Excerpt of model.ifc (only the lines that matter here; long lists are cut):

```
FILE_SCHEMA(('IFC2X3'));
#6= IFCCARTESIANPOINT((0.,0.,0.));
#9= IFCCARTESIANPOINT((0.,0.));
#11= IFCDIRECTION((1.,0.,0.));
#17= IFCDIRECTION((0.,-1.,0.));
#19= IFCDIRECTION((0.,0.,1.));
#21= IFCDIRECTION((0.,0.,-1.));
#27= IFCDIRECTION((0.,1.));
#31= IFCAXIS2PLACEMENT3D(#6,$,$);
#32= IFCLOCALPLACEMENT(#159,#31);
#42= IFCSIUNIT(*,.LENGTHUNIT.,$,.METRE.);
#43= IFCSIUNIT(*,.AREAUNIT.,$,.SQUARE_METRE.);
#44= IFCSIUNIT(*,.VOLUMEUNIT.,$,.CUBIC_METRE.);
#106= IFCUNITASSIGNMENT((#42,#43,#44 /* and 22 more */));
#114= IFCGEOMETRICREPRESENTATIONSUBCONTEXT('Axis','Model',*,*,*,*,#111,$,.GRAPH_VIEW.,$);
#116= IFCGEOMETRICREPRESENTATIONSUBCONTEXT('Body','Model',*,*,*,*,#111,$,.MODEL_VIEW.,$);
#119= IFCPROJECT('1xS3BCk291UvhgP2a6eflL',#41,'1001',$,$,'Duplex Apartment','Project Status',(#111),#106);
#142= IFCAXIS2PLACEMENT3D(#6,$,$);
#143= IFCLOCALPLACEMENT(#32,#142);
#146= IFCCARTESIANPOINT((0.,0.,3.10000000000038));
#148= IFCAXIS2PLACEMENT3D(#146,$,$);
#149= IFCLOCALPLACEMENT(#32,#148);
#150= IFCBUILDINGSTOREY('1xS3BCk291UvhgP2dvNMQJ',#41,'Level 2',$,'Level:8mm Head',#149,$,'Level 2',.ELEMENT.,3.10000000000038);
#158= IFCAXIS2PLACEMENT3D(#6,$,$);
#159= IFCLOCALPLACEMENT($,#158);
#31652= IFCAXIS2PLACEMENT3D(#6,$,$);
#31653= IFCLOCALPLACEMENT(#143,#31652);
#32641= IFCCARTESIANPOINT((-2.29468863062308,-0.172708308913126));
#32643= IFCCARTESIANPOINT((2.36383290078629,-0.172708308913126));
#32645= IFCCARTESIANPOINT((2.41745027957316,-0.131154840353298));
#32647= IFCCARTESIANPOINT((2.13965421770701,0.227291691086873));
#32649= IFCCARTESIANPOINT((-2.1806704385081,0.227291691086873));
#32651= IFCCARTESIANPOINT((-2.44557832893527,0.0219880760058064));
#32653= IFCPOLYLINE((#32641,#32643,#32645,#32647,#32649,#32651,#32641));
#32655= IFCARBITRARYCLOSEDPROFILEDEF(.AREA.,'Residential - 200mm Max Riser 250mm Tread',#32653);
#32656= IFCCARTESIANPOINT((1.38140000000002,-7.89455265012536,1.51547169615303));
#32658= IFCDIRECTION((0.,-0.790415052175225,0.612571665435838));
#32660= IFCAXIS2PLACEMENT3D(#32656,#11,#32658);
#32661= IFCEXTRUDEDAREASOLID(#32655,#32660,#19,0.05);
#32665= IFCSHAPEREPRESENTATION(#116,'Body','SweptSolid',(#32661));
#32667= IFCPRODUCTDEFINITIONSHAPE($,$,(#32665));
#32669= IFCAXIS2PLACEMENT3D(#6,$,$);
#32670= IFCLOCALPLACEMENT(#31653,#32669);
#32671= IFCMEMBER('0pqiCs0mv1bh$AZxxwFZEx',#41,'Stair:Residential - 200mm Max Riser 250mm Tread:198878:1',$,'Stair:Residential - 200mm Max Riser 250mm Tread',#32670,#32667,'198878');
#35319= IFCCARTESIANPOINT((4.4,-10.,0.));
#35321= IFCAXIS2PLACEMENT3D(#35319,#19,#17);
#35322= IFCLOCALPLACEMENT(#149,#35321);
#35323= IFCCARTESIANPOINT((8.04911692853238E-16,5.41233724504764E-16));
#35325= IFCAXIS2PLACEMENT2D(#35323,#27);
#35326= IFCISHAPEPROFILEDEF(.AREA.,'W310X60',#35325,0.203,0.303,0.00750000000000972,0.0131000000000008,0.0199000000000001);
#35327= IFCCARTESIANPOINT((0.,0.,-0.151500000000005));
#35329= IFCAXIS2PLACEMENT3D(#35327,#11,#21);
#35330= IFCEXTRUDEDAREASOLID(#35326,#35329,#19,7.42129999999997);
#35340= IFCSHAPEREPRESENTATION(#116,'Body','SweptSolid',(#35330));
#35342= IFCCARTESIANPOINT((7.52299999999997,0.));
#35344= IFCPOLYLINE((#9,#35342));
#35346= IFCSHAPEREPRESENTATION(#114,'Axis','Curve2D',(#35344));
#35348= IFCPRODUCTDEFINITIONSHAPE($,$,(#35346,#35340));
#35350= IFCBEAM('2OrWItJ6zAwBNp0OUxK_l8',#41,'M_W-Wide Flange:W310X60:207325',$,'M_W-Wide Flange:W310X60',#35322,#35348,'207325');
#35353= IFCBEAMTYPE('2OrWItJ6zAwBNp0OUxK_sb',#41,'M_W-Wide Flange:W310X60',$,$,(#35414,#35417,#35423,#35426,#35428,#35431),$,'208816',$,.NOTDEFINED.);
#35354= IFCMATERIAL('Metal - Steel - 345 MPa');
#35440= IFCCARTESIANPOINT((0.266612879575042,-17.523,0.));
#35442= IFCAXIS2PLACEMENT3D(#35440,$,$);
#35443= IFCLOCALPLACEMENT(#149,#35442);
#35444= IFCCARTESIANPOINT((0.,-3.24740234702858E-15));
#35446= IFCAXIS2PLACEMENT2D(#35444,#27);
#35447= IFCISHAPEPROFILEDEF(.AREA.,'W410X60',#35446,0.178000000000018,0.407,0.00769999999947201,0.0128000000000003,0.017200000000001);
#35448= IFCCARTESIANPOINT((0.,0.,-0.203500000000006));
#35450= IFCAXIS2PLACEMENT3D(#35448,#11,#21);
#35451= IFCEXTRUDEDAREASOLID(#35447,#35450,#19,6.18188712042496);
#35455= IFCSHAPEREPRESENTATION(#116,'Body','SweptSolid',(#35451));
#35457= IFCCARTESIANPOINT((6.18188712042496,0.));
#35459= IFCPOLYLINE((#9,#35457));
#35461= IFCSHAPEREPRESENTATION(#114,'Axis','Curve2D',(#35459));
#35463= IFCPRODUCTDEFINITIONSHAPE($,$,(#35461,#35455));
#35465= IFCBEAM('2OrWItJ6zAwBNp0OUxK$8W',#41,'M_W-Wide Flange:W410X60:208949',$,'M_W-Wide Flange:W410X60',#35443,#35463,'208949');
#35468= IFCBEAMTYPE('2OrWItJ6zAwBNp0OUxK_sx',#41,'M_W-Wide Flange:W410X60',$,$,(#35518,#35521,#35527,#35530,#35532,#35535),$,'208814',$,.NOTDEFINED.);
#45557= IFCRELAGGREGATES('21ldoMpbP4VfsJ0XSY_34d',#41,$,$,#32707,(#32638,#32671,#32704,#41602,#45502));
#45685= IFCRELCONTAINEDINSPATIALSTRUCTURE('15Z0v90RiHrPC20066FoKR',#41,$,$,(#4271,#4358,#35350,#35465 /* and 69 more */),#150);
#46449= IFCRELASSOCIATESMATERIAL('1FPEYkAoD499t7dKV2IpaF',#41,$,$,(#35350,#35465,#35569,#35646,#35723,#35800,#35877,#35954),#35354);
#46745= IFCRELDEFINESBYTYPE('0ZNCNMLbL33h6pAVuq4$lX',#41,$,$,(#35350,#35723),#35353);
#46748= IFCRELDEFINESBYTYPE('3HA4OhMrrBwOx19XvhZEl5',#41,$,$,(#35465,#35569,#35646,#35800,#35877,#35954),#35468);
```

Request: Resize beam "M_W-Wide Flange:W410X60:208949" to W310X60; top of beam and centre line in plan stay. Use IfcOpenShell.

```python
import ifcopenshell
import ifcopenshell.api.type
import ifcopenshell.util.element
import ifcopenshell.util.representation

model = ifcopenshell.open("model.ifc")

member = model.by_guid("2OrWItJ6zAwBNp0OUxK$8W")
source = next(p for p in model.by_type("IfcIShapeProfileDef") if p.ProfileName == "W310X60")

body = ifcopenshell.util.representation.get_representation(member, "Model", "Body")
solid = body.Items[0]
old_profile = solid.SweptArea

# Copy the section's sizes but keep this member's own profile position.
profile = ifcopenshell.util.element.copy(model, source)
# Profiles are centred, so shift by half the change in depth to hold the top.
shift = (old_profile.OverallDepth - profile.OverallDepth) / 2
x, y = old_profile.Position.Location.Coordinates
up = (-1.0, 0.0)  # upwards, in the solid's own plane
location = model.createIfcCartesianPoint((x + up[0] * shift, y + up[1] * shift))
profile.Position = model.createIfcAxis2Placement2D(location, old_profile.Position.RefDirection)
solid.SweptArea = profile
if not model.get_total_inverses(old_profile):
    ifcopenshell.util.element.remove_deep2(model, old_profile)

new_type = model.by_id(35353)
ifcopenshell.api.type.assign_type(
    model, related_objects=[member], relating_type=new_type, should_map_representations=False
)
member.Name = member.Name.replace("W410X60", "W310X60")
member.ObjectType = "M_W-Wide Flange:W310X60"

print(solid.SweptArea)

model.write("model_v2.ifc")
```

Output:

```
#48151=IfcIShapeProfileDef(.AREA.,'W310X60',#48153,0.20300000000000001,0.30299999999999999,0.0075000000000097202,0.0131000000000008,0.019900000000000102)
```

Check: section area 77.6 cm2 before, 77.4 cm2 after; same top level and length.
